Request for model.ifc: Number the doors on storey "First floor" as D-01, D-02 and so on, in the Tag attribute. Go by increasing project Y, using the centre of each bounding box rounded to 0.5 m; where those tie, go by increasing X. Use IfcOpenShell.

First a look at what the model holds.

```python
import ifcopenshell
import ifcopenshell.util.element
import ifcopenshell.util.placement

model = ifcopenshell.open("model.ifc")
print(model.schema)
storey = next(s for s in model.by_type("IfcBuildingStorey") if s.Name == "First floor")
doors = [e for e in ifcopenshell.util.element.get_decomposition(storey) if e.is_a("IfcDoor")]
for e in sorted(doors, key=lambda e: e.id()):
    origin = ifcopenshell.util.placement.get_local_placement(e.ObjectPlacement)[:3, 3]
    print(e.id(), e.Tag, e.Name, origin.round(2) + 0.0, sep=" | ")
```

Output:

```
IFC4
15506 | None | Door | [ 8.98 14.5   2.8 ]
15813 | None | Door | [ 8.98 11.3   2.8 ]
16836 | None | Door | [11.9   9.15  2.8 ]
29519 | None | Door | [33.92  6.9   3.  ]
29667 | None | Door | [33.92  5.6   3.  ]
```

```python
import ifcopenshell
import ifcopenshell.geom
import ifcopenshell.util.element
import ifcopenshell.util.shape

model = ifcopenshell.open("model.ifc")
settings = ifcopenshell.geom.settings()
settings.set("use-world-coords", True)


def centre(element):
    shape = ifcopenshell.geom.create_shape(settings, element)
    return ifcopenshell.util.shape.get_bbox_centroid(shape.geometry)


storey = next(s for s in model.by_type("IfcBuildingStorey") if s.Name == "First floor")
doors = [e for e in ifcopenshell.util.element.get_decomposition(storey) if e.is_a("IfcDoor")]

# Insertion points can sit at a corner or the storey origin, so sort by the geometry (in metres).
centres = {e: centre(e) for e in doors}
doors.sort(key=lambda e: (round(centres[e][1] / 0.5), centres[e][0]))

for i, e in enumerate(doors, start=1):
    number = f"D-{i:02d}"
    e.Tag = number
    print(e.id(), number)

model.write("model_v2.ifc")
```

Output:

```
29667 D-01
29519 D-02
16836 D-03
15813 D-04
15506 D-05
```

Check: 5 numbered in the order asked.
